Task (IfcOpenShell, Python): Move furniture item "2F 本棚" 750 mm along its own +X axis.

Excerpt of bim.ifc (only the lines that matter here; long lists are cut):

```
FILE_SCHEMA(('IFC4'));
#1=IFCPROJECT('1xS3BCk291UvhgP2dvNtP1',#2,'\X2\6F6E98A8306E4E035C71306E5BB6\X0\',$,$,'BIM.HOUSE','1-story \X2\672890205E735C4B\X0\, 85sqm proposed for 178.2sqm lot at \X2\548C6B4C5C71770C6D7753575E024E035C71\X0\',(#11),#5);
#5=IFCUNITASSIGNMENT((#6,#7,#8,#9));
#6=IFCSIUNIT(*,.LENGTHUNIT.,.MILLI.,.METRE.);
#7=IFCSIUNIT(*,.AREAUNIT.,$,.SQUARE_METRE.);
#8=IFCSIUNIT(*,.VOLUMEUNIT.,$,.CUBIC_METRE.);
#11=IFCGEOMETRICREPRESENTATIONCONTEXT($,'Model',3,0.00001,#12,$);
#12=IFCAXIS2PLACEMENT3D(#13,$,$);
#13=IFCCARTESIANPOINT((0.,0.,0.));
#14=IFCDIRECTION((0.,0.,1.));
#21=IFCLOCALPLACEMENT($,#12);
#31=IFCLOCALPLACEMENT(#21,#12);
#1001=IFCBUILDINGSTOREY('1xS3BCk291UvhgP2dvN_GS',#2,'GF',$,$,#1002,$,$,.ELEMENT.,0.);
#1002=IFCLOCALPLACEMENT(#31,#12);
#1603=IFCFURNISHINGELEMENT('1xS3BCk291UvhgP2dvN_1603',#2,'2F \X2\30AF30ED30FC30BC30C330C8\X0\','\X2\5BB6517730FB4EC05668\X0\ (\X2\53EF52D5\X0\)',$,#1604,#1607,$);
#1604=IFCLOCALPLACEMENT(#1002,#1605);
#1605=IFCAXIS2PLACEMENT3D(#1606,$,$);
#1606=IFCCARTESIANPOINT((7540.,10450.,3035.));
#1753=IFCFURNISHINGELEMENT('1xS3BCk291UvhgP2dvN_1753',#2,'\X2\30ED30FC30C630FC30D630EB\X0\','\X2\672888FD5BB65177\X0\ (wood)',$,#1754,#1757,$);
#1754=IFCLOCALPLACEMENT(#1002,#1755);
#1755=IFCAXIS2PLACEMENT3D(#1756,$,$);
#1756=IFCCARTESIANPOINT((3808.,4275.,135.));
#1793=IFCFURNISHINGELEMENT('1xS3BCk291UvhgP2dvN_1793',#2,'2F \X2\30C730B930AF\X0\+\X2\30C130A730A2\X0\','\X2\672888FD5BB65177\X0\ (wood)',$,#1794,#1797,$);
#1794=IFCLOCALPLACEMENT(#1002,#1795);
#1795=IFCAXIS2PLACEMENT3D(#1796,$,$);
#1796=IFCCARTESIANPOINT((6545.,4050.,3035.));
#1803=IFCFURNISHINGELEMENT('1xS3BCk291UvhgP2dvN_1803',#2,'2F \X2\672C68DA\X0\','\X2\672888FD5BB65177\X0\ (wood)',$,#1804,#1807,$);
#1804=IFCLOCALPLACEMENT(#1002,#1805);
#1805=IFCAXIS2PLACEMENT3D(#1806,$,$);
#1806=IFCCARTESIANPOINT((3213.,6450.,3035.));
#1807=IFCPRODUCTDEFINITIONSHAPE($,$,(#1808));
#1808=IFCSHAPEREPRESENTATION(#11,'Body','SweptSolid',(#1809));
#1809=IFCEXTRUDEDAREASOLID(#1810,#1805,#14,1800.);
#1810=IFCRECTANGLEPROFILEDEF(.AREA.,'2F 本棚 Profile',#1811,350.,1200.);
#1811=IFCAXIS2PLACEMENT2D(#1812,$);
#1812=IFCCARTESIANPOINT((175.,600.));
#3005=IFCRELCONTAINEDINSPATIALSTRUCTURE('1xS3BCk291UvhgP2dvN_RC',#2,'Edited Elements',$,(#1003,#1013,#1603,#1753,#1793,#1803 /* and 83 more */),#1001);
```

```python
import ifcopenshell
import ifcopenshell.api.geometry
import ifcopenshell.util.placement
import ifcopenshell.util.unit

model = ifcopenshell.open("bim.ifc")
unit_scale = ifcopenshell.util.unit.calculate_unit_scale(model)

item = model.by_guid("1xS3BCk291UvhgP2dvN_1803")
matrix = ifcopenshell.util.placement.get_local_placement(item.ObjectPlacement)
matrix[:3, 3] += matrix[:3, 0] * 0.75 / unit_scale
ifcopenshell.api.geometry.edit_object_placement(model, product=item, matrix=matrix, is_si=False)

print(ifcopenshell.util.placement.get_local_placement(item.ObjectPlacement).round(3) + 0.0)

model.write("bim_rev.ifc")
```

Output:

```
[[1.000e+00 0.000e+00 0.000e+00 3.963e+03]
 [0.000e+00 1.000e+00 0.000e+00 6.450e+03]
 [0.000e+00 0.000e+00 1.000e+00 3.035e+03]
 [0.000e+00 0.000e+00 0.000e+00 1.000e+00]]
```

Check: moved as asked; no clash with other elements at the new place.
